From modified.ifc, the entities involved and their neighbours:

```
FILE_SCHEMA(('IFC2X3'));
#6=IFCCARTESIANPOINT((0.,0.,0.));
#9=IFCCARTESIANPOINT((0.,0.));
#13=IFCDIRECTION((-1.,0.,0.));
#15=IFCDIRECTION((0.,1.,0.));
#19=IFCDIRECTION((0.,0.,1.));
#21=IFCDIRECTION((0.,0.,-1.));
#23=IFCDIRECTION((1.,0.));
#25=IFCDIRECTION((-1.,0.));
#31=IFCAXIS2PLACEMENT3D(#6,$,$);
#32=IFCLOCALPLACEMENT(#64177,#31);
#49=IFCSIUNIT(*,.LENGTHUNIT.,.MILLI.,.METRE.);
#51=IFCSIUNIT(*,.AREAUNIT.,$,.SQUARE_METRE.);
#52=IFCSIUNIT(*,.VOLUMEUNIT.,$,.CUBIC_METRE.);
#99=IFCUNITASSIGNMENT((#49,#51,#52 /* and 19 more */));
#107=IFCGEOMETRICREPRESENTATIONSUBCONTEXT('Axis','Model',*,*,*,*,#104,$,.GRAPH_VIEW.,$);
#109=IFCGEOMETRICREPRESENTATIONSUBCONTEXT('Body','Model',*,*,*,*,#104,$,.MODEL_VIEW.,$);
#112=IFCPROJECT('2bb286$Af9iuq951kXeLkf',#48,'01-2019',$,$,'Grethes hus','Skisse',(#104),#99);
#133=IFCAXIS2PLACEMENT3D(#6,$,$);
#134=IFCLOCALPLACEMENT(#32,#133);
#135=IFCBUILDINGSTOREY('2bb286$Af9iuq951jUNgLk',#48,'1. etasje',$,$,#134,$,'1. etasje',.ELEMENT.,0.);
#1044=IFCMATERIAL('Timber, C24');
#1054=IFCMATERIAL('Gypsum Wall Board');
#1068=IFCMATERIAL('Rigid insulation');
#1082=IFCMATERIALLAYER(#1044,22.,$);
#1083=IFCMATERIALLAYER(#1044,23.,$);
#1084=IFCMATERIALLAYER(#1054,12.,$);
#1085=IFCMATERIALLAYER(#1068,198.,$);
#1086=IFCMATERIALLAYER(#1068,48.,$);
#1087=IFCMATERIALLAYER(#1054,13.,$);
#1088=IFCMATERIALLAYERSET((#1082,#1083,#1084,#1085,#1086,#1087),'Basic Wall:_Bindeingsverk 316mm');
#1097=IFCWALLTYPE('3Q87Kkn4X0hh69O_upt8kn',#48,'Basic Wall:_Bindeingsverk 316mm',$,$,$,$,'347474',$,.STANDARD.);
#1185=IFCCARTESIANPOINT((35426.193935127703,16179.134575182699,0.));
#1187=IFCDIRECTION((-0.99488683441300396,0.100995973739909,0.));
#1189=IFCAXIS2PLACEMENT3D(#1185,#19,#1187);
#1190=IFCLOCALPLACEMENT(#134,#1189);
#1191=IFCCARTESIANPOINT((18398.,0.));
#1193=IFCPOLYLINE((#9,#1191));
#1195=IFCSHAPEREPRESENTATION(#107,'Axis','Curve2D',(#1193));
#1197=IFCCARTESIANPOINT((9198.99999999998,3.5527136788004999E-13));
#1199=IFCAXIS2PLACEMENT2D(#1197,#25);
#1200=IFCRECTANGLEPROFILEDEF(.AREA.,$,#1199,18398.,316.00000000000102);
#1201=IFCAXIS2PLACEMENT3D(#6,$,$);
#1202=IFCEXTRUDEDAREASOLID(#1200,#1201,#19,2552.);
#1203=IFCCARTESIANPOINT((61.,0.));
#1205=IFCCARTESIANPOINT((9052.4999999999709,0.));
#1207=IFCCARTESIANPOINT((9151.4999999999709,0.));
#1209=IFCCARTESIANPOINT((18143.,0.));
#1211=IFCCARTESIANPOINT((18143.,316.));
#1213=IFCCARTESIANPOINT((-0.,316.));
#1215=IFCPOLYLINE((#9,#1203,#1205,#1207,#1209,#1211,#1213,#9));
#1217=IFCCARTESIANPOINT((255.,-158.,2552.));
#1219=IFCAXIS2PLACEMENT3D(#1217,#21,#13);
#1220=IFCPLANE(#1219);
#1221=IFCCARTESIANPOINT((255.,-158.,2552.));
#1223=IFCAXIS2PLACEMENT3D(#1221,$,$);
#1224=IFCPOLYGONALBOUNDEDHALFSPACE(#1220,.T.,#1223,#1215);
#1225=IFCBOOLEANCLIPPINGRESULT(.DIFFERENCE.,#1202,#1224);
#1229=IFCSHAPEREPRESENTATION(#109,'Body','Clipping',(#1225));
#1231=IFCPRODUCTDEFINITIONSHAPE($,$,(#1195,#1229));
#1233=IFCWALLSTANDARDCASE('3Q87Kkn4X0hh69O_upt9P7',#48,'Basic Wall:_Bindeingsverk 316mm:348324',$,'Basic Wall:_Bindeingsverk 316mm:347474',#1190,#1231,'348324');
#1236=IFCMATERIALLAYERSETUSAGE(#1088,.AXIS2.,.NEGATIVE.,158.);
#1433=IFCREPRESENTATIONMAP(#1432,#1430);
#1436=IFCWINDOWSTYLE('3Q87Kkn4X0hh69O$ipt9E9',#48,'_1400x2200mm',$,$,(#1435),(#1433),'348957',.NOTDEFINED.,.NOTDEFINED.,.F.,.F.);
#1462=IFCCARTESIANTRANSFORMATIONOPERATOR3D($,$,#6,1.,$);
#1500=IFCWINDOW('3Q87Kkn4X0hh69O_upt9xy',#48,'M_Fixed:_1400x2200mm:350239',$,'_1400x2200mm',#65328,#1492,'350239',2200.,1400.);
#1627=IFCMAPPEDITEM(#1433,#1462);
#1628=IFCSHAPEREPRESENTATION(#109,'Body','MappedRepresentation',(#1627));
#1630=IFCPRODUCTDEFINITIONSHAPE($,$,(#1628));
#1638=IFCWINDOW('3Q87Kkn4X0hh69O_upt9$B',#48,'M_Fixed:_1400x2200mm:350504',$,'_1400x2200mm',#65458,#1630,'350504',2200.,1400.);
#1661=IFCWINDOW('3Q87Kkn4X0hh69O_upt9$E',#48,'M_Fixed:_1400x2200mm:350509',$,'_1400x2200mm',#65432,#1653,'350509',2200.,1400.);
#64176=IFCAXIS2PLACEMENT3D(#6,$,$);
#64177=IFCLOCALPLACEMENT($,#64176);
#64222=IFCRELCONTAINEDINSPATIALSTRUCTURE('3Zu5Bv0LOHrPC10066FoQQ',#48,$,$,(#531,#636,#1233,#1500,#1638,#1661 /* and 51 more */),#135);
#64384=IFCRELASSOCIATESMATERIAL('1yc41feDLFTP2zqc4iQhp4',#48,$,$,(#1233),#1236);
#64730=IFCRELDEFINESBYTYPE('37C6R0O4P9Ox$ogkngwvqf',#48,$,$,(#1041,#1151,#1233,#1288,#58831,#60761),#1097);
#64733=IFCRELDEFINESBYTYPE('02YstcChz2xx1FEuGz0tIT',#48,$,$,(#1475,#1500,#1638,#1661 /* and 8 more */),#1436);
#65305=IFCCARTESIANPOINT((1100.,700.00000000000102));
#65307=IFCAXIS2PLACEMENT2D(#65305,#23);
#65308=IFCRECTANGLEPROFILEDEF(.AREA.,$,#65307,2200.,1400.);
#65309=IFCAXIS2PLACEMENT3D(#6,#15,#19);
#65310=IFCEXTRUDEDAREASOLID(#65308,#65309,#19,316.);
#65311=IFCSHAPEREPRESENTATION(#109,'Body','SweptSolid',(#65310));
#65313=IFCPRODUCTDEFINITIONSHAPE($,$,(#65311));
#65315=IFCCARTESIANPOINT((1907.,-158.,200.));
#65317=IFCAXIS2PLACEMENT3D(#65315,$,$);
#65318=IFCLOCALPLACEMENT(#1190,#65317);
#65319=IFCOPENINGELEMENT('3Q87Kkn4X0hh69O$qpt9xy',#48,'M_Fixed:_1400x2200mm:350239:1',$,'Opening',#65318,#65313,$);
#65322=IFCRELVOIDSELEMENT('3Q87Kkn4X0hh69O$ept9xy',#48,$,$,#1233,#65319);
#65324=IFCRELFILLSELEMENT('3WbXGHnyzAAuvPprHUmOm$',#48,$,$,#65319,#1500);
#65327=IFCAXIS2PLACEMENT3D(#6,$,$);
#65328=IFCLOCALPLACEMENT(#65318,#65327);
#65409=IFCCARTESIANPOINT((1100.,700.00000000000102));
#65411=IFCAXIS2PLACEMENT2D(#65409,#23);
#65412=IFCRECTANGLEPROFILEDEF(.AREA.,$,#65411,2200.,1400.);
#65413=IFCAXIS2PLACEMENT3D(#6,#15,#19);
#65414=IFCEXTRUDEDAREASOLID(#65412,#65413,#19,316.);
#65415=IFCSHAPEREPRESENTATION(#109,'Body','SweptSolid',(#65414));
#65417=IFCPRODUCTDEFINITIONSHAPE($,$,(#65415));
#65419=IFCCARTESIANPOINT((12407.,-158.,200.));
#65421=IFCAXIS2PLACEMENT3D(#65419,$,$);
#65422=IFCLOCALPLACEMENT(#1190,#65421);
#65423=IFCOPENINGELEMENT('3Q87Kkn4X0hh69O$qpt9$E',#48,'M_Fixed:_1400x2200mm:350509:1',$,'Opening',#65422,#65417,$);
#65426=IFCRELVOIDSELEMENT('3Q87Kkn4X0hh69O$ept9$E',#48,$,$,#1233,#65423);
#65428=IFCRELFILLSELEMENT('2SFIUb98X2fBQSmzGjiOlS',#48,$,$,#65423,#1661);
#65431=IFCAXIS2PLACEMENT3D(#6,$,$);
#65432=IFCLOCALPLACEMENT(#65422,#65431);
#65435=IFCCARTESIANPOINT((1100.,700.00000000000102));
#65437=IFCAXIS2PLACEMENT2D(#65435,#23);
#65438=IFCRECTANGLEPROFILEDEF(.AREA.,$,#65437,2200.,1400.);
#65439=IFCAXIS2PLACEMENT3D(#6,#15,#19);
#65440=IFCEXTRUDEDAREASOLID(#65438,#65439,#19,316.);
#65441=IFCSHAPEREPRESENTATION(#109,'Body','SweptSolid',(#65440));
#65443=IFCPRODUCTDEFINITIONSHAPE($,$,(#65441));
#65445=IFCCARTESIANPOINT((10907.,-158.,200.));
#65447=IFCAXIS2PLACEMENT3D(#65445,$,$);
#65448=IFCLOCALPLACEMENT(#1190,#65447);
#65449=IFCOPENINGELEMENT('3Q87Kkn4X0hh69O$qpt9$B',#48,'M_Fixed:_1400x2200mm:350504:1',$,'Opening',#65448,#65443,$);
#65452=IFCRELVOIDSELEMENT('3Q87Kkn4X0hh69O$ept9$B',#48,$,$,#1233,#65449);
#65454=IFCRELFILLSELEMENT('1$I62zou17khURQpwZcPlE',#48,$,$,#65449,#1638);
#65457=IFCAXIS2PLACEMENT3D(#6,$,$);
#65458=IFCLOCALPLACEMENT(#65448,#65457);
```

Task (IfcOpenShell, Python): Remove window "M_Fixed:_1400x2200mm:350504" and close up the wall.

```python
import ifcopenshell
import ifcopenshell.api.feature
import ifcopenshell.api.root
import ifcopenshell.geom
import ifcopenshell.util.shape

model = ifcopenshell.open("modified.ifc")
settings = ifcopenshell.geom.settings()


def volume(element):
    """Net volume in cubic metres, openings subtracted."""
    shape = ifcopenshell.geom.create_shape(settings, element)
    return ifcopenshell.util.shape.get_volume(shape.geometry)


window = model.by_id(1638)
opening = window.FillsVoids[0].RelatingOpeningElement
wall = opening.VoidsElements[0].RelatingBuildingElement
before = volume(wall)

ifcopenshell.api.root.remove_product(model, product=window)
ifcopenshell.api.feature.remove_feature(model, feature=opening)

after = volume(wall)

print(f"wall volume {before:.3f} -> {after:.3f} m3")

model.write("modified-out.ifc")
```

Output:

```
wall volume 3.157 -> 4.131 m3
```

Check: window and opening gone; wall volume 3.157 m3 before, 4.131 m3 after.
